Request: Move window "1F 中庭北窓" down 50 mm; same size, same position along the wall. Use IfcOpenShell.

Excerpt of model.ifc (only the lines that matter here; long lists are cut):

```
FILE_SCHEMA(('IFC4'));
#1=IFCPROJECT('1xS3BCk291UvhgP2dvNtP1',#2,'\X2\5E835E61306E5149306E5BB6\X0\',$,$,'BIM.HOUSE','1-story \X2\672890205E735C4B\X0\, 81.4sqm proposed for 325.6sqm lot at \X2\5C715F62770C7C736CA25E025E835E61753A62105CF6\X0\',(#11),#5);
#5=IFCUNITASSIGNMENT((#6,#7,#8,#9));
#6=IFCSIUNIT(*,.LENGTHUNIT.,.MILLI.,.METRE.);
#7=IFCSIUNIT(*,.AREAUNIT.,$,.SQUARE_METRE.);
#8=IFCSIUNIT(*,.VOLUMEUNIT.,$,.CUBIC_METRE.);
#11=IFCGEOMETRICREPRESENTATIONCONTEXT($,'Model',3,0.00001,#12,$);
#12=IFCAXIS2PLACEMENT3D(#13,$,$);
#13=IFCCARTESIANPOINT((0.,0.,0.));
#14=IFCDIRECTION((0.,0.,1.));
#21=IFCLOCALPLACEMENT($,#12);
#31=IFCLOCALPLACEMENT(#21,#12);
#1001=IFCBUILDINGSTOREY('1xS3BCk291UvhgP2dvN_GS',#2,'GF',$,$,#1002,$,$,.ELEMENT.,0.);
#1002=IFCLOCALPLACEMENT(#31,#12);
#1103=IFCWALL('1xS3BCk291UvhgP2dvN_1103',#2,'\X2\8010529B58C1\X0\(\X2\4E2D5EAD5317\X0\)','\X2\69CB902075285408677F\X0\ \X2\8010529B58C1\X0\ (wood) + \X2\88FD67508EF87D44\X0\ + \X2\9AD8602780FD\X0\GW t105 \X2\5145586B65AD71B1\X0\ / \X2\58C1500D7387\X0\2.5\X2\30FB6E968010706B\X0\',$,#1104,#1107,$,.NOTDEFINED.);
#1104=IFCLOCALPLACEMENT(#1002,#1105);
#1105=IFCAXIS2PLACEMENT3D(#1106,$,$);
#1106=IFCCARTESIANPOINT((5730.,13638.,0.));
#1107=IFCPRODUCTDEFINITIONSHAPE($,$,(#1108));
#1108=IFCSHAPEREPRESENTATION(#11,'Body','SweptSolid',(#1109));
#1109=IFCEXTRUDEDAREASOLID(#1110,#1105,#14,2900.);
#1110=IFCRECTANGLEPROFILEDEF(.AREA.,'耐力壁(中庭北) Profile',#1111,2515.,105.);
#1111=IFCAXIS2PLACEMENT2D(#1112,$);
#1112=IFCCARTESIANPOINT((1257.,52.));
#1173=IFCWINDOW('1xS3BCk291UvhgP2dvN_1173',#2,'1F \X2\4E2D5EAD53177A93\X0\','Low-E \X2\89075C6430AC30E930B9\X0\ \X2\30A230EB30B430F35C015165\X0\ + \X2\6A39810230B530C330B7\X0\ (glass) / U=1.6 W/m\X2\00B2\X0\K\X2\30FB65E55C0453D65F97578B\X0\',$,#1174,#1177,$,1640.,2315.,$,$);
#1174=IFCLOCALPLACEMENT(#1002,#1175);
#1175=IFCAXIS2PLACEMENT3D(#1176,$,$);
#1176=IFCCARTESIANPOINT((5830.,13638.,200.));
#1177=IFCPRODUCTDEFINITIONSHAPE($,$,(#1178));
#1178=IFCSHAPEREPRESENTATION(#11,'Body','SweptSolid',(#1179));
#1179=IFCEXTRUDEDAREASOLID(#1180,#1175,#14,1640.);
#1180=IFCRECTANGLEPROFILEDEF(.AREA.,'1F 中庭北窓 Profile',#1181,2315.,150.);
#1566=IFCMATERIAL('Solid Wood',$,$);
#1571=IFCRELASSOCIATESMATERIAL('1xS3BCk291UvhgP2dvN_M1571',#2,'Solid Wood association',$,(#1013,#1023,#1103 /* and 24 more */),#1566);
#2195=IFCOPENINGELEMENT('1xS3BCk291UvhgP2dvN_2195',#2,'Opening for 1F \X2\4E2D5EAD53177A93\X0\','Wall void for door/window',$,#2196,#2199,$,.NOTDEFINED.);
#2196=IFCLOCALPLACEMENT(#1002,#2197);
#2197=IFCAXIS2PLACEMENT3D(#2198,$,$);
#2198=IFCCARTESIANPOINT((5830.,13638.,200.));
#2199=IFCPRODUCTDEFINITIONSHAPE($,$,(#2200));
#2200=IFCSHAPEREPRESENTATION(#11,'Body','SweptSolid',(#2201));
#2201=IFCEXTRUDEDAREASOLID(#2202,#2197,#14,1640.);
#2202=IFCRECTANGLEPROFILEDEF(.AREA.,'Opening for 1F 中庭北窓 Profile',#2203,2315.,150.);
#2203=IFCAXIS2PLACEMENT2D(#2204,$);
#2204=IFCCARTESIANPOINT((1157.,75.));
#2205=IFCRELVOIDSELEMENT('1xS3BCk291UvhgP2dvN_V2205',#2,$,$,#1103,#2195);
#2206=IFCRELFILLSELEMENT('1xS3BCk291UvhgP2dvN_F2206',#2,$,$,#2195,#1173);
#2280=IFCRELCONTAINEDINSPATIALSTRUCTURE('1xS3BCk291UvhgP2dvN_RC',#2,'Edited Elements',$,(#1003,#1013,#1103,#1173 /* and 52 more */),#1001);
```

```python
import numpy as np
import ifcopenshell
import ifcopenshell.api.geometry
import ifcopenshell.util.placement
import ifcopenshell.util.unit

model = ifcopenshell.open("model.ifc")
unit_scale = ifcopenshell.util.unit.calculate_unit_scale(model)

window = model.by_guid("1xS3BCk291UvhgP2dvN_1173")
opening = window.FillsVoids[0].RelatingOpeningElement
dz = -0.05 / unit_scale

shift = np.array([0.0, 0.0, dz])
# The window is not placed relative to its opening, so move both.
for product in (opening, window):
    matrix = ifcopenshell.util.placement.get_local_placement(product.ObjectPlacement)
    matrix[:3, 3] += shift
    ifcopenshell.api.geometry.edit_object_placement(model, product=product, matrix=matrix, is_si=False)

print(f"moved by {dz * unit_scale:+.3f} m")

model.write("model_rev.ifc")
```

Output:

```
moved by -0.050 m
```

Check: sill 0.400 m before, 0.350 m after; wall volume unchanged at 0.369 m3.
